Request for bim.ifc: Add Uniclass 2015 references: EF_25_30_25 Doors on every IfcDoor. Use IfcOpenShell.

First a look at what the model holds.

```python
import ifcopenshell

model = ifcopenshell.open("bim.ifc")
print(model.schema)
print("classifications:", [c.Name for c in model.by_type("IfcClassification")])
for ifc_class in ("IfcDoor", "IfcRoof", "IfcStair", "IfcWall", "IfcWindow"):
    print(ifc_class, len(model.by_type(ifc_class)))
```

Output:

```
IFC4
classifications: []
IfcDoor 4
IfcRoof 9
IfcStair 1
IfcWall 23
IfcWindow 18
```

```python
import ifcopenshell
import ifcopenshell.api.classification

model = ifcopenshell.open("bim.ifc")

system = ifcopenshell.api.classification.add_classification(model, classification="Uniclass 2015")

codes = {
    "IfcDoor": ("EF_25_30_25", "Doors"),
}
for ifc_class, (code, name) in codes.items():
    products = model.by_type(ifc_class)
    ifcopenshell.api.classification.add_reference(
        model, products=products, classification=system, identification=code, name=name
    )
    print(code, len(products))

model.write("bim_updated.ifc")
```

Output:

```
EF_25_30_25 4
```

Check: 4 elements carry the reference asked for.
